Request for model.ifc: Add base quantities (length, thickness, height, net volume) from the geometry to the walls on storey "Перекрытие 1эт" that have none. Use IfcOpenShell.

First a look at what the model holds.

```python
import ifcopenshell
import ifcopenshell.util.element
import ifcopenshell.util.unit

model = ifcopenshell.open("model.ifc")
print(model.schema)
for unit_type in ("LENGTHUNIT", "AREAUNIT", "VOLUMEUNIT"):
    print(unit_type, ifcopenshell.util.unit.calculate_unit_scale(model, unit_type))
storey = next(s for s in model.by_type("IfcBuildingStorey") if s.Name == "Перекрытие 1эт")
walls = [e for e in ifcopenshell.util.element.get_decomposition(storey) if e.is_a("IfcWall")]
for e in sorted(walls, key=lambda e: e.id()):
    print(e.id(), e.is_a(), e.Name, list(ifcopenshell.util.element.get_psets(e, qtos_only=True)), sep=" | ")
```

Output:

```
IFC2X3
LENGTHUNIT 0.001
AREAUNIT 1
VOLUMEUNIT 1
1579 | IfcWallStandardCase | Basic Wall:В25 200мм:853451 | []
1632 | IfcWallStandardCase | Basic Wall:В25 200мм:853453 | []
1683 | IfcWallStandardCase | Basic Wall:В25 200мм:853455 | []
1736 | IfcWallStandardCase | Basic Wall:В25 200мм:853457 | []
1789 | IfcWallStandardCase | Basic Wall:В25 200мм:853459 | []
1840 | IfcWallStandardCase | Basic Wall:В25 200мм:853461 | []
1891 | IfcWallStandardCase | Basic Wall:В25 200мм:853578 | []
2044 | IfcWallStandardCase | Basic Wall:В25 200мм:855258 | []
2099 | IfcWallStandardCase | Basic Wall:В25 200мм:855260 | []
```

```python
import ifcopenshell
import ifcopenshell.api.pset
import ifcopenshell.geom
import ifcopenshell.util.element
import ifcopenshell.util.shape
import ifcopenshell.util.unit

model = ifcopenshell.open("model.ifc")
unit_scale = ifcopenshell.util.unit.calculate_unit_scale(model)
volume_scale = ifcopenshell.util.unit.calculate_unit_scale(model, "VOLUMEUNIT")
settings = ifcopenshell.geom.settings()

storey = next(s for s in model.by_type("IfcBuildingStorey") if s.Name == "Перекрытие 1эт")
walls = [e for e in ifcopenshell.util.element.get_decomposition(storey) if e.is_a("IfcWall")]

for e in sorted(walls, key=lambda e: e.id()):
    if ifcopenshell.util.element.get_psets(e, qtos_only=True, should_inherit=False):
        continue
    # Geometry comes back in metres, in the element's own axes.
    shape = ifcopenshell.geom.create_shape(settings, e)
    values = {
        "Length": ifcopenshell.util.shape.get_x(shape.geometry) / unit_scale,
        "Width": ifcopenshell.util.shape.get_y(shape.geometry) / unit_scale,
        "Height": ifcopenshell.util.shape.get_z(shape.geometry) / unit_scale,
        "NetVolume": ifcopenshell.util.shape.get_volume(shape.geometry) / volume_scale,
    }
    qto = ifcopenshell.api.pset.add_qto(model, product=e, name="BaseQuantities")
    ifcopenshell.api.pset.edit_qto(model, qto=qto, properties=values)
    print(e.id(), {k: round(v, 3) for k, v in values.items()})

model.write("model_updated.ifc")
```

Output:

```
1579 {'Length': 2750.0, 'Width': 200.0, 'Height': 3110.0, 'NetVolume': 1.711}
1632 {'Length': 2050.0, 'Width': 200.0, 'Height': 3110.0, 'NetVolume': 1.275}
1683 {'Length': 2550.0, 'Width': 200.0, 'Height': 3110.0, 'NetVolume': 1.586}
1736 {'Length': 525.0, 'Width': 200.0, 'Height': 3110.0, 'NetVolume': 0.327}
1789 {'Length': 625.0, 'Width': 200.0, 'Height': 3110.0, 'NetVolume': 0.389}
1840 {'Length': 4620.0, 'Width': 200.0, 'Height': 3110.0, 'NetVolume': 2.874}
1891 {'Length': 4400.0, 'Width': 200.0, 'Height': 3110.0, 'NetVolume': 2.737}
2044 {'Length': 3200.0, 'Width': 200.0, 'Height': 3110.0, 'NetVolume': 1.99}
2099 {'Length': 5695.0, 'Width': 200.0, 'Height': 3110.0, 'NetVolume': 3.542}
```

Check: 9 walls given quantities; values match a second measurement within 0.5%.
